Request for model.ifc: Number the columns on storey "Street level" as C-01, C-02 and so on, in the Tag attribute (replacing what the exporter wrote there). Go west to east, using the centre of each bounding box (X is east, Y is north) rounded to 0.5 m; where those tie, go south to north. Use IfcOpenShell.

First a look at what the model holds.

```python
import ifcopenshell
import ifcopenshell.util.element
import ifcopenshell.util.placement

model = ifcopenshell.open("model.ifc")
print(model.schema)
storey = next(s for s in model.by_type("IfcBuildingStorey") if s.Name == "Street level")
columns = [e for e in ifcopenshell.util.element.get_decomposition(storey) if e.is_a("IfcColumn")]
for e in sorted(columns, key=lambda e: e.id()):
    origin = ifcopenshell.util.placement.get_local_placement(e.ObjectPlacement)[:3, 3]
    print(e.id(), e.Tag, e.Name, origin.round(2) + 0.0, sep=" | ")
```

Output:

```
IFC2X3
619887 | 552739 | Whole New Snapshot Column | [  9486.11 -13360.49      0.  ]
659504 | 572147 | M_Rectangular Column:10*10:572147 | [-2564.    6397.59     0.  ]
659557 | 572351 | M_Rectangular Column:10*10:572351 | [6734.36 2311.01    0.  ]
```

```python
import ifcopenshell
import ifcopenshell.geom
import ifcopenshell.util.element
import ifcopenshell.util.shape

model = ifcopenshell.open("model.ifc")
settings = ifcopenshell.geom.settings()
settings.set("use-world-coords", True)


def centre(element):
    shape = ifcopenshell.geom.create_shape(settings, element)
    return ifcopenshell.util.shape.get_bbox_centroid(shape.geometry)


storey = next(s for s in model.by_type("IfcBuildingStorey") if s.Name == "Street level")
columns = [e for e in ifcopenshell.util.element.get_decomposition(storey) if e.is_a("IfcColumn")]

# Insertion points can sit at a corner or the storey origin, so sort by the geometry (in metres).
centres = {e: centre(e) for e in columns}
columns.sort(key=lambda e: (round(centres[e][0] / 0.5), centres[e][1]))

for i, e in enumerate(columns, start=1):
    number = f"C-{i:02d}"
    e.Tag = number
    print(e.id(), number)

model.write("model_updated.ifc")
```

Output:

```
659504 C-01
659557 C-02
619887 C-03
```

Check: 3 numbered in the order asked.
